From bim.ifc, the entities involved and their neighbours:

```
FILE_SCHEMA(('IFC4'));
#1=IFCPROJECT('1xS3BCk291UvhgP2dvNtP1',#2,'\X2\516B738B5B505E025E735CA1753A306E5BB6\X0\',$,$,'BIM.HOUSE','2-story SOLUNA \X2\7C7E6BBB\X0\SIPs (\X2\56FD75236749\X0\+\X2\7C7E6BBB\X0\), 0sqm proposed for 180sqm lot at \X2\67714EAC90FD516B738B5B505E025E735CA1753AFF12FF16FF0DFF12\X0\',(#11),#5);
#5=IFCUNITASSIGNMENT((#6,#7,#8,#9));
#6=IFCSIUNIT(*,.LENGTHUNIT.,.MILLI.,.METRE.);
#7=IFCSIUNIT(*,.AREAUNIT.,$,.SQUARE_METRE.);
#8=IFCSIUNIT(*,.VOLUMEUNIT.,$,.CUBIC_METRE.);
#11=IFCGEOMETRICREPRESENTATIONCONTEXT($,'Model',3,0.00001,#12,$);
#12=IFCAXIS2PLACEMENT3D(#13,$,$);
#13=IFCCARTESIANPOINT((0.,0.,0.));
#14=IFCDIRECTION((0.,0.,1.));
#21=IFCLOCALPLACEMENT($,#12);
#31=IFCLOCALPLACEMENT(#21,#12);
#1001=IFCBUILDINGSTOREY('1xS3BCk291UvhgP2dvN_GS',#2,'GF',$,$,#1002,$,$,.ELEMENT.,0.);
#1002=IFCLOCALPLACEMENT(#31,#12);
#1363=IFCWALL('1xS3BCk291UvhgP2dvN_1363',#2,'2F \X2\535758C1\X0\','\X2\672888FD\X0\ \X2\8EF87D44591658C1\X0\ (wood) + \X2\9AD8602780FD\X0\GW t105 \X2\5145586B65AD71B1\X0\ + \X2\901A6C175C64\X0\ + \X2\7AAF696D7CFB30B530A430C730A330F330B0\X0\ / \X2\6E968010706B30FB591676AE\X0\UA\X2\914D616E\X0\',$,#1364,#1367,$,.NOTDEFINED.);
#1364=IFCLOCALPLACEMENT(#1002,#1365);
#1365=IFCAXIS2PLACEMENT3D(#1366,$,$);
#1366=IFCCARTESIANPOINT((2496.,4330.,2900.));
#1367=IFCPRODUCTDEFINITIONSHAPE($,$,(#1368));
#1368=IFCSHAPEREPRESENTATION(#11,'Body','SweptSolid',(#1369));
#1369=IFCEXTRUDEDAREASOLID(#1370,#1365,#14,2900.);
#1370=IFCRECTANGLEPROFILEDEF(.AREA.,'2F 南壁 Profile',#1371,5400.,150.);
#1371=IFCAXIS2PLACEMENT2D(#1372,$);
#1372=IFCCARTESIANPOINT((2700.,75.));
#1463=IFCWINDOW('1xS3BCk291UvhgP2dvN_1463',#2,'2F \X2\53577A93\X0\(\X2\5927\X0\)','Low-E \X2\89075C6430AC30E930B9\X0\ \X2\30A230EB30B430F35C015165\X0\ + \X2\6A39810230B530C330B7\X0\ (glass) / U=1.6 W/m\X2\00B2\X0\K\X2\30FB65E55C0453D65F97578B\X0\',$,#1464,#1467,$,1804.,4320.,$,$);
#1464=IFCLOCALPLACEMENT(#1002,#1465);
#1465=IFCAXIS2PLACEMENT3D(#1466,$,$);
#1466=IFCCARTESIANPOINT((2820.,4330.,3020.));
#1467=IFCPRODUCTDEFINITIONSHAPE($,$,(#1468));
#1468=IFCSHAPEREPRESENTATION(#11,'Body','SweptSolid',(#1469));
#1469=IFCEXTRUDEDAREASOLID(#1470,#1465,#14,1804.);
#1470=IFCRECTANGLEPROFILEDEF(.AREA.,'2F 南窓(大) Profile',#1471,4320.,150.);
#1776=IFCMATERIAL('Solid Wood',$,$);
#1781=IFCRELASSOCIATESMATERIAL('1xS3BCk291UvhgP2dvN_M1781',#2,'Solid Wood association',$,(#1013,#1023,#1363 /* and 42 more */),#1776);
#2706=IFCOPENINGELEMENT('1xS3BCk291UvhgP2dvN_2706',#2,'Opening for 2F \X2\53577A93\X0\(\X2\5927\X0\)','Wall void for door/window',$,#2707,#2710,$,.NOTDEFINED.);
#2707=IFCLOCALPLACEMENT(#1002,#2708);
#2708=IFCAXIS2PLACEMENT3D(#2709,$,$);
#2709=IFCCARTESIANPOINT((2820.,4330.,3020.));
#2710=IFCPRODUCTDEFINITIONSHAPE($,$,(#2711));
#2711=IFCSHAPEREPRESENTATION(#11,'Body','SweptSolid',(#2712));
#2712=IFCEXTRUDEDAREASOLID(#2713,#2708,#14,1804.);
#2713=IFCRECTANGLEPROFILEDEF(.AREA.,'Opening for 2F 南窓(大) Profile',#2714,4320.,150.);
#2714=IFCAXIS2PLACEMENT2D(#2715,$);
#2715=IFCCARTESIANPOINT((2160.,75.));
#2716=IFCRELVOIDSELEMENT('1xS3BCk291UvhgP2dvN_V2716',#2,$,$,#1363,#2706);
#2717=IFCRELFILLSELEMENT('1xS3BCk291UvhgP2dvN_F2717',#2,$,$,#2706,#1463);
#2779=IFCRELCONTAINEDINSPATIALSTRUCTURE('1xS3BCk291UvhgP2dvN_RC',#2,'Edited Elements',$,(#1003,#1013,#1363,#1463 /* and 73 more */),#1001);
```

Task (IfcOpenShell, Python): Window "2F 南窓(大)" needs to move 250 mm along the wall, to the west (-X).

```python
import ifcopenshell
import ifcopenshell.api.geometry
import ifcopenshell.util.placement

model = ifcopenshell.open("bim.ifc")

window = model.by_id(1463)
opening = window.FillsVoids[0].RelatingOpeningElement
wall = opening.VoidsElements[0].RelatingBuildingElement

wall_matrix = ifcopenshell.util.placement.get_local_placement(wall.ObjectPlacement)
shift = wall_matrix[:3, 0] * -250.0
before = ifcopenshell.util.placement.get_local_placement(window.ObjectPlacement)[:3, 3].copy()

# The window is not placed relative to its opening, so move both.
for product in (opening, window):
    matrix = ifcopenshell.util.placement.get_local_placement(product.ObjectPlacement)
    matrix[:3, 3] += shift
    ifcopenshell.api.geometry.edit_object_placement(model, product=product, matrix=matrix, is_si=False)

after = ifcopenshell.util.placement.get_local_placement(window.ObjectPlacement)[:3, 3]
print("window moved by", (after - before).round(3) + 0.0)

model.write("bim_edited.ifc")
```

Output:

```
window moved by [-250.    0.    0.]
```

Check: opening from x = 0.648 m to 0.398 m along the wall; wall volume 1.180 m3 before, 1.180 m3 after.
